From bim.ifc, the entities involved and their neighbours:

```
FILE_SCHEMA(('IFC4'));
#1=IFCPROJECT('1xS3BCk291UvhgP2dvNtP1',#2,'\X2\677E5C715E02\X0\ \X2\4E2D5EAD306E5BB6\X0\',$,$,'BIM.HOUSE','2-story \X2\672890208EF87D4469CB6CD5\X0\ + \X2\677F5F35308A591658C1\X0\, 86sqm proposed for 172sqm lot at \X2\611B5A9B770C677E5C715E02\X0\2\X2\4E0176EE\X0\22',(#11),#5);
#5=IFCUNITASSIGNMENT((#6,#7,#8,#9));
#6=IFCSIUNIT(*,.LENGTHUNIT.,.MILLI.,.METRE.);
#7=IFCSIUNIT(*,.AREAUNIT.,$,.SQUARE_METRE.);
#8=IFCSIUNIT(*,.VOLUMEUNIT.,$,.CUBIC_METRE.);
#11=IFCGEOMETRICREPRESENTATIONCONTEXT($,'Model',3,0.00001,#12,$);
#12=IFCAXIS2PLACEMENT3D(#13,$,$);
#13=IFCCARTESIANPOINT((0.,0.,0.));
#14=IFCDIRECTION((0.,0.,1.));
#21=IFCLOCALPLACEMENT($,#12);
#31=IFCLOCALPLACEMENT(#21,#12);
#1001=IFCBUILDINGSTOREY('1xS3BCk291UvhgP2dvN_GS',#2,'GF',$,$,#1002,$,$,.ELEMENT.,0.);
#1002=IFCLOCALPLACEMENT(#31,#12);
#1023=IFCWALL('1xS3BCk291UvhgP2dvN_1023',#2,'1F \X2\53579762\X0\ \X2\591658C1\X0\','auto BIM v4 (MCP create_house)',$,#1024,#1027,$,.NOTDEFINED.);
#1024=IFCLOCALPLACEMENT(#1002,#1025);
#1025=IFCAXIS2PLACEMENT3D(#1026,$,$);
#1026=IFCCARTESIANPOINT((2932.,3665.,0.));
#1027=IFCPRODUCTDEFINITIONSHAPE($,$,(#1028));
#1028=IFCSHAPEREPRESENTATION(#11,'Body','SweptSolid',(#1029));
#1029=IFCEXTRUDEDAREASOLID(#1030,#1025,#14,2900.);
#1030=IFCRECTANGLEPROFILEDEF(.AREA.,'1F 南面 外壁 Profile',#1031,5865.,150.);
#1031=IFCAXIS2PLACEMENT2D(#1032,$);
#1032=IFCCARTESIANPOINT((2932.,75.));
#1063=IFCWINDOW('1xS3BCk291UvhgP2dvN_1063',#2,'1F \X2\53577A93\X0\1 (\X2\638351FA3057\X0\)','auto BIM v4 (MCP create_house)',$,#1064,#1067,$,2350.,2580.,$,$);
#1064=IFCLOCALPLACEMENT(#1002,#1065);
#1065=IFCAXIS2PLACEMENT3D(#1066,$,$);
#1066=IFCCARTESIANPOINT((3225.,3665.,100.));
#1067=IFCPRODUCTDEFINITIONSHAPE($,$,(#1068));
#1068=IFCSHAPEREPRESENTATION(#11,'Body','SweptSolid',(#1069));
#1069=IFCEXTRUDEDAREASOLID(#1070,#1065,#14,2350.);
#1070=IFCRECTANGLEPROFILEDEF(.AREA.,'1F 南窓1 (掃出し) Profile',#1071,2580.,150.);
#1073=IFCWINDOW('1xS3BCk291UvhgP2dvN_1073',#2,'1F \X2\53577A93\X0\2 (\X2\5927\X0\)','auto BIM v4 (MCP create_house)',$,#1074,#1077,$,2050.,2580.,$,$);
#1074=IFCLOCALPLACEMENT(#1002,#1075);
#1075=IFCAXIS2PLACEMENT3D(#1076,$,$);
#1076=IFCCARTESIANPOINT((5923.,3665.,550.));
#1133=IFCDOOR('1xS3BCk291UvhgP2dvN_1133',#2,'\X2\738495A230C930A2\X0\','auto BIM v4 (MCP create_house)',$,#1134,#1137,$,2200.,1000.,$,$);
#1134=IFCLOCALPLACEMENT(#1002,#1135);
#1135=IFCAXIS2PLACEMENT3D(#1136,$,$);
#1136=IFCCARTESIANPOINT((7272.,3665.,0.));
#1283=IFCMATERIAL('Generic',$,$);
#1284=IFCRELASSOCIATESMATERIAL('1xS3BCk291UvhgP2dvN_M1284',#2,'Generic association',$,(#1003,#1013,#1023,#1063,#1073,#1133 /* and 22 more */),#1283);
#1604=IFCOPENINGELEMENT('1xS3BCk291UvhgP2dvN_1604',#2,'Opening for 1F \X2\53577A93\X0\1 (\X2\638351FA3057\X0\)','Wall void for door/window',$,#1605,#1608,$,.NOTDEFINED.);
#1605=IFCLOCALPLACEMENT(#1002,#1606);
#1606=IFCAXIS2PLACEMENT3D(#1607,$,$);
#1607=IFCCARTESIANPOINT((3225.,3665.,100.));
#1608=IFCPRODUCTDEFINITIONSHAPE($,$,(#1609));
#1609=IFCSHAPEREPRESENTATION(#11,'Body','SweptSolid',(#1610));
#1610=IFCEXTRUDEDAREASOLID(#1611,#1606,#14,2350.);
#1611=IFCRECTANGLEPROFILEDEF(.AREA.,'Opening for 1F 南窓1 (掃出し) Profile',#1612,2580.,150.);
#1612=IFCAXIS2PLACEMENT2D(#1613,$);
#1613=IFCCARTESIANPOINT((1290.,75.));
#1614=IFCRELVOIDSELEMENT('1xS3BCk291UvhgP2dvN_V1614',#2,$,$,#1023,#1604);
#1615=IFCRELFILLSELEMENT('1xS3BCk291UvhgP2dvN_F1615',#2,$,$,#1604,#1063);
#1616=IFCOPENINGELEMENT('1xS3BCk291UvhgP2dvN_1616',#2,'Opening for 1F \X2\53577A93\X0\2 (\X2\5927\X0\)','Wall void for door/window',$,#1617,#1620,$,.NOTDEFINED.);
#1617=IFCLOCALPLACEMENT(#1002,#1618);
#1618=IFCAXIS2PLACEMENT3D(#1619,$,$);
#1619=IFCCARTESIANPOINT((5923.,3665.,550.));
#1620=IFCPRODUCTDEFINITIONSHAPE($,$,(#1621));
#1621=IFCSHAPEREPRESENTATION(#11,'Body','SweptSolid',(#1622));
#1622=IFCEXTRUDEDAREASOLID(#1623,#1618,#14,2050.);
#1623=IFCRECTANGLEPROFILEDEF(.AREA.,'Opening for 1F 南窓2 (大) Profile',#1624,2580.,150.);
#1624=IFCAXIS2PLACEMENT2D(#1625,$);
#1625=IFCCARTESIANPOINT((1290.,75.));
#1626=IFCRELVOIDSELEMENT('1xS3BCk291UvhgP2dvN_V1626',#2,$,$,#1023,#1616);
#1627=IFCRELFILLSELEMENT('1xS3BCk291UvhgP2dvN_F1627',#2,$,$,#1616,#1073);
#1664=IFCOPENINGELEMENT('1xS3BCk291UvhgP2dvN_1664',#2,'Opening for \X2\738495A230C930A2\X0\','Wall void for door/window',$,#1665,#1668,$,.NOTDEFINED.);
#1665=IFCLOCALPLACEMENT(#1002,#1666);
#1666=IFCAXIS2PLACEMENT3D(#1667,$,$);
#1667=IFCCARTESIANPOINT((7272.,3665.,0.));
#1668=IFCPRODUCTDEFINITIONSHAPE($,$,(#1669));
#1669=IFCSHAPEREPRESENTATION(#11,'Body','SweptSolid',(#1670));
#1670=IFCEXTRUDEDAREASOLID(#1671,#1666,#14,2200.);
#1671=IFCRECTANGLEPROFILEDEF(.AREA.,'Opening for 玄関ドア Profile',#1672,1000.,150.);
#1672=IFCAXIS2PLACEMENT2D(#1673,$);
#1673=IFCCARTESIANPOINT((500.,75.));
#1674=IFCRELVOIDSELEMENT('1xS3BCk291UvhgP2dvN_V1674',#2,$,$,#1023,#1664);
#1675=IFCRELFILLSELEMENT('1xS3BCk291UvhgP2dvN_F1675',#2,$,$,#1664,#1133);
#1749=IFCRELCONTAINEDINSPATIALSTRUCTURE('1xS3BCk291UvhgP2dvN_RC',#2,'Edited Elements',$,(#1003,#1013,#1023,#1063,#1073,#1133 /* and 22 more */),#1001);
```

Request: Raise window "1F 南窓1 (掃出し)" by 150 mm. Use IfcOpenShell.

```python
import numpy as np
import ifcopenshell
import ifcopenshell.api.geometry
import ifcopenshell.util.placement
import ifcopenshell.util.unit

model = ifcopenshell.open("bim.ifc")
unit_scale = ifcopenshell.util.unit.calculate_unit_scale(model)

window = model.by_id(1063)
opening = window.FillsVoids[0].RelatingOpeningElement
dz = 0.15 / unit_scale

shift = np.array([0.0, 0.0, dz])
# The window is not placed relative to its opening, so move both.
for product in (opening, window):
    matrix = ifcopenshell.util.placement.get_local_placement(product.ObjectPlacement)
    matrix[:3, 3] += shift
    ifcopenshell.api.geometry.edit_object_placement(model, product=product, matrix=matrix, is_si=False)

print(f"moved by {dz * unit_scale:+.3f} m")

model.write("bim_edited.ifc")
```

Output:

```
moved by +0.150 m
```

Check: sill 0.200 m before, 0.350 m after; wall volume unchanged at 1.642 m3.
